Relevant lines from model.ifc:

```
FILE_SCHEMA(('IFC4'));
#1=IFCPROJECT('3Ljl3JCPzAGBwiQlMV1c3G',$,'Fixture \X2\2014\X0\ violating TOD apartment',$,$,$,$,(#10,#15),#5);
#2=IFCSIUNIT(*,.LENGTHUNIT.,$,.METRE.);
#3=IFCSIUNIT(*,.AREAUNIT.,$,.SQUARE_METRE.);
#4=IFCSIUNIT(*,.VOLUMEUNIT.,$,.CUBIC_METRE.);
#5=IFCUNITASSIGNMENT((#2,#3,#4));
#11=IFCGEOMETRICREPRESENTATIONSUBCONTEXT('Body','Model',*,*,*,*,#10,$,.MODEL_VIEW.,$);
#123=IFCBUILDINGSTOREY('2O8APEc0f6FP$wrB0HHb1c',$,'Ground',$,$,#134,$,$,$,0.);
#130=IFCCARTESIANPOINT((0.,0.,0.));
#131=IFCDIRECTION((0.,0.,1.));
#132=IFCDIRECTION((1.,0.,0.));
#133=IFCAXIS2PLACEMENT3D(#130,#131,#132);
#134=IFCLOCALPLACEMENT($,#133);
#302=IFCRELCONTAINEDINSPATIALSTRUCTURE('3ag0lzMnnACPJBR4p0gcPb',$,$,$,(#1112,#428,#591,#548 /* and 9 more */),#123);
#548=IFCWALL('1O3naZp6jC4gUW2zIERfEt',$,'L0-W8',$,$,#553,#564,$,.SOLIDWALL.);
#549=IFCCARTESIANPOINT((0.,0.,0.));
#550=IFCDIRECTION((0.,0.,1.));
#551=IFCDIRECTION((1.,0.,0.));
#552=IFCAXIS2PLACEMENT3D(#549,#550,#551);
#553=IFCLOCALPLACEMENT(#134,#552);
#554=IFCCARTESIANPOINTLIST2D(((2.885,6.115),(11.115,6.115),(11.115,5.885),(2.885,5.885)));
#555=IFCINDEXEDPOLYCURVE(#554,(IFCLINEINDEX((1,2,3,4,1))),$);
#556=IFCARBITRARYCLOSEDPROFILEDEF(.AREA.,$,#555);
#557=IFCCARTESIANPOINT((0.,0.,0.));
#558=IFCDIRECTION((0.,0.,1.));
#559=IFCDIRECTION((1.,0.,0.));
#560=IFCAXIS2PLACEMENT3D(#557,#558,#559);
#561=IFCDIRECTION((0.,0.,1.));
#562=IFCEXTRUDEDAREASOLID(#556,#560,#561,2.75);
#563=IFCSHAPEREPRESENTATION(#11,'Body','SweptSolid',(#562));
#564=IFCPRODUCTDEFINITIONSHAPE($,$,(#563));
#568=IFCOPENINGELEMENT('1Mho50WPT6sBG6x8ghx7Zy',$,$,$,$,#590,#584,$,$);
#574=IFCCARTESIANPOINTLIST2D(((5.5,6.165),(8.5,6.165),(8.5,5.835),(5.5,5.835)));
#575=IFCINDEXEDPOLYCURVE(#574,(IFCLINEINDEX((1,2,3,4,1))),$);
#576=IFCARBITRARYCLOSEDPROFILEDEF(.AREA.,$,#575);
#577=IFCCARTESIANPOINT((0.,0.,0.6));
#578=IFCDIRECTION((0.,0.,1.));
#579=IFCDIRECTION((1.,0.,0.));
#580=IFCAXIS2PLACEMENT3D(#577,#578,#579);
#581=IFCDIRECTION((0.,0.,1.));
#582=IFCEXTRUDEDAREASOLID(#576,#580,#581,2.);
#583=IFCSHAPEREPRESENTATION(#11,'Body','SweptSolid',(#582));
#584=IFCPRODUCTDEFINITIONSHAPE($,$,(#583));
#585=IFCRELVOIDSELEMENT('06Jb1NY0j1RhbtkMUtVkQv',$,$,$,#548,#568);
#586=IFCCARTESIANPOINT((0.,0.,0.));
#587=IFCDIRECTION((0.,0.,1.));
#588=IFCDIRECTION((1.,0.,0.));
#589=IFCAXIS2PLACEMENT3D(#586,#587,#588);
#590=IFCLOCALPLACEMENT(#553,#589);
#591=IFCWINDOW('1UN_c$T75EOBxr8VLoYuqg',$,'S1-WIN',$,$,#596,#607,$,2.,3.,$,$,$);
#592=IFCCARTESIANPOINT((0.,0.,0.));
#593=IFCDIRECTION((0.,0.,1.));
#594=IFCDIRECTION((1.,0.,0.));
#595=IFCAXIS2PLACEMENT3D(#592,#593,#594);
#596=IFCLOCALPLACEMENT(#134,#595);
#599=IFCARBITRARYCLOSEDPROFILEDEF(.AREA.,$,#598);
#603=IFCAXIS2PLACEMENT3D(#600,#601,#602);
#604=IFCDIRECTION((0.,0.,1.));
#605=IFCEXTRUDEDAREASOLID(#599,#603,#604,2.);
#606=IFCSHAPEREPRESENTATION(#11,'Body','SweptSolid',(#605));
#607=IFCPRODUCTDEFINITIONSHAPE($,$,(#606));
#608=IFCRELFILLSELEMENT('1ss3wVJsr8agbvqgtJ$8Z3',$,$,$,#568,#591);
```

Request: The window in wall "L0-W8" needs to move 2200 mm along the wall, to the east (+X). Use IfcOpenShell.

```python
import ifcopenshell
import ifcopenshell.api.geometry
import ifcopenshell.util.placement

model = ifcopenshell.open("model.ifc")

window = model.by_guid("1UN_c$T75EOBxr8VLoYuqg")
opening = window.FillsVoids[0].RelatingOpeningElement
wall = opening.VoidsElements[0].RelatingBuildingElement

wall_matrix = ifcopenshell.util.placement.get_local_placement(wall.ObjectPlacement)
shift = wall_matrix[:3, 0] * 2.2
before = ifcopenshell.util.placement.get_local_placement(window.ObjectPlacement)[:3, 3].copy()

# The window is not placed relative to its opening, so move both.
for product in (opening, window):
    matrix = ifcopenshell.util.placement.get_local_placement(product.ObjectPlacement)
    matrix[:3, 3] += shift
    ifcopenshell.api.geometry.edit_object_placement(model, product=product, matrix=matrix, is_si=False)

after = ifcopenshell.util.placement.get_local_placement(window.ObjectPlacement)[:3, 3]
print("window moved by", (after - before).round(3) + 0.0)

model.write("model_v2.ifc")
```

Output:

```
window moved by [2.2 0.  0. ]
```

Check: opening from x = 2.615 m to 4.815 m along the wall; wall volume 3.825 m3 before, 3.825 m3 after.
